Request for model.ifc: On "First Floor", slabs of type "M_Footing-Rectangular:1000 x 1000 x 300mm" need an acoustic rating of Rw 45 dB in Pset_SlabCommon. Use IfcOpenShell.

First a look at what the model holds.

```python
import ifcopenshell
import ifcopenshell.util.element

model = ifcopenshell.open("model.ifc")
print(model.schema)
storey = next(s for s in model.by_type("IfcBuildingStorey") if s.Name == "First Floor")
slabs = [e for e in ifcopenshell.util.element.get_decomposition(storey) if e.is_a("IfcSlab")]
seen = {}
for e in slabs:
    element_type = ifcopenshell.util.element.get_type(e)
    key = (element_type.Name if element_type != e and element_type else None, ifcopenshell.util.element.get_pset(e, "Pset_SlabCommon", "AcousticRating"))
    seen[key] = seen.get(key, 0) + 1
for (name, value), count in sorted(seen.items(), key=str):
    print(count, "x", name, "|", value)
```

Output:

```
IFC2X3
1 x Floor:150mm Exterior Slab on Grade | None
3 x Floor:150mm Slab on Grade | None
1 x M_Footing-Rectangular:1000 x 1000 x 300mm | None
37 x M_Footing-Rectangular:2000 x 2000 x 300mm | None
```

```python
import ifcopenshell
import ifcopenshell.api.pset
import ifcopenshell.util.element

model = ifcopenshell.open("model.ifc")

storey = next(s for s in model.by_type("IfcBuildingStorey") if s.Name == "First Floor")
slabs = [e for e in ifcopenshell.util.element.get_decomposition(storey) if e.is_a("IfcSlab")]

count = 0
for e in slabs:
    element_type = ifcopenshell.util.element.get_type(e)
    if element_type in (None, e) or element_type.Name != "M_Footing-Rectangular:1000 x 1000 x 300mm":
        continue
    # add_pset returns the element's existing set when there is one.
    pset = ifcopenshell.api.pset.add_pset(model, product=e, name="Pset_SlabCommon")
    ifcopenshell.api.pset.edit_pset(model, pset=pset, properties={"AcousticRating": "Rw 45 dB"})
    count += 1

print(count, "slabs updated")

model.write("model-out.ifc")
```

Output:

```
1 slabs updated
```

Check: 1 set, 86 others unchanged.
